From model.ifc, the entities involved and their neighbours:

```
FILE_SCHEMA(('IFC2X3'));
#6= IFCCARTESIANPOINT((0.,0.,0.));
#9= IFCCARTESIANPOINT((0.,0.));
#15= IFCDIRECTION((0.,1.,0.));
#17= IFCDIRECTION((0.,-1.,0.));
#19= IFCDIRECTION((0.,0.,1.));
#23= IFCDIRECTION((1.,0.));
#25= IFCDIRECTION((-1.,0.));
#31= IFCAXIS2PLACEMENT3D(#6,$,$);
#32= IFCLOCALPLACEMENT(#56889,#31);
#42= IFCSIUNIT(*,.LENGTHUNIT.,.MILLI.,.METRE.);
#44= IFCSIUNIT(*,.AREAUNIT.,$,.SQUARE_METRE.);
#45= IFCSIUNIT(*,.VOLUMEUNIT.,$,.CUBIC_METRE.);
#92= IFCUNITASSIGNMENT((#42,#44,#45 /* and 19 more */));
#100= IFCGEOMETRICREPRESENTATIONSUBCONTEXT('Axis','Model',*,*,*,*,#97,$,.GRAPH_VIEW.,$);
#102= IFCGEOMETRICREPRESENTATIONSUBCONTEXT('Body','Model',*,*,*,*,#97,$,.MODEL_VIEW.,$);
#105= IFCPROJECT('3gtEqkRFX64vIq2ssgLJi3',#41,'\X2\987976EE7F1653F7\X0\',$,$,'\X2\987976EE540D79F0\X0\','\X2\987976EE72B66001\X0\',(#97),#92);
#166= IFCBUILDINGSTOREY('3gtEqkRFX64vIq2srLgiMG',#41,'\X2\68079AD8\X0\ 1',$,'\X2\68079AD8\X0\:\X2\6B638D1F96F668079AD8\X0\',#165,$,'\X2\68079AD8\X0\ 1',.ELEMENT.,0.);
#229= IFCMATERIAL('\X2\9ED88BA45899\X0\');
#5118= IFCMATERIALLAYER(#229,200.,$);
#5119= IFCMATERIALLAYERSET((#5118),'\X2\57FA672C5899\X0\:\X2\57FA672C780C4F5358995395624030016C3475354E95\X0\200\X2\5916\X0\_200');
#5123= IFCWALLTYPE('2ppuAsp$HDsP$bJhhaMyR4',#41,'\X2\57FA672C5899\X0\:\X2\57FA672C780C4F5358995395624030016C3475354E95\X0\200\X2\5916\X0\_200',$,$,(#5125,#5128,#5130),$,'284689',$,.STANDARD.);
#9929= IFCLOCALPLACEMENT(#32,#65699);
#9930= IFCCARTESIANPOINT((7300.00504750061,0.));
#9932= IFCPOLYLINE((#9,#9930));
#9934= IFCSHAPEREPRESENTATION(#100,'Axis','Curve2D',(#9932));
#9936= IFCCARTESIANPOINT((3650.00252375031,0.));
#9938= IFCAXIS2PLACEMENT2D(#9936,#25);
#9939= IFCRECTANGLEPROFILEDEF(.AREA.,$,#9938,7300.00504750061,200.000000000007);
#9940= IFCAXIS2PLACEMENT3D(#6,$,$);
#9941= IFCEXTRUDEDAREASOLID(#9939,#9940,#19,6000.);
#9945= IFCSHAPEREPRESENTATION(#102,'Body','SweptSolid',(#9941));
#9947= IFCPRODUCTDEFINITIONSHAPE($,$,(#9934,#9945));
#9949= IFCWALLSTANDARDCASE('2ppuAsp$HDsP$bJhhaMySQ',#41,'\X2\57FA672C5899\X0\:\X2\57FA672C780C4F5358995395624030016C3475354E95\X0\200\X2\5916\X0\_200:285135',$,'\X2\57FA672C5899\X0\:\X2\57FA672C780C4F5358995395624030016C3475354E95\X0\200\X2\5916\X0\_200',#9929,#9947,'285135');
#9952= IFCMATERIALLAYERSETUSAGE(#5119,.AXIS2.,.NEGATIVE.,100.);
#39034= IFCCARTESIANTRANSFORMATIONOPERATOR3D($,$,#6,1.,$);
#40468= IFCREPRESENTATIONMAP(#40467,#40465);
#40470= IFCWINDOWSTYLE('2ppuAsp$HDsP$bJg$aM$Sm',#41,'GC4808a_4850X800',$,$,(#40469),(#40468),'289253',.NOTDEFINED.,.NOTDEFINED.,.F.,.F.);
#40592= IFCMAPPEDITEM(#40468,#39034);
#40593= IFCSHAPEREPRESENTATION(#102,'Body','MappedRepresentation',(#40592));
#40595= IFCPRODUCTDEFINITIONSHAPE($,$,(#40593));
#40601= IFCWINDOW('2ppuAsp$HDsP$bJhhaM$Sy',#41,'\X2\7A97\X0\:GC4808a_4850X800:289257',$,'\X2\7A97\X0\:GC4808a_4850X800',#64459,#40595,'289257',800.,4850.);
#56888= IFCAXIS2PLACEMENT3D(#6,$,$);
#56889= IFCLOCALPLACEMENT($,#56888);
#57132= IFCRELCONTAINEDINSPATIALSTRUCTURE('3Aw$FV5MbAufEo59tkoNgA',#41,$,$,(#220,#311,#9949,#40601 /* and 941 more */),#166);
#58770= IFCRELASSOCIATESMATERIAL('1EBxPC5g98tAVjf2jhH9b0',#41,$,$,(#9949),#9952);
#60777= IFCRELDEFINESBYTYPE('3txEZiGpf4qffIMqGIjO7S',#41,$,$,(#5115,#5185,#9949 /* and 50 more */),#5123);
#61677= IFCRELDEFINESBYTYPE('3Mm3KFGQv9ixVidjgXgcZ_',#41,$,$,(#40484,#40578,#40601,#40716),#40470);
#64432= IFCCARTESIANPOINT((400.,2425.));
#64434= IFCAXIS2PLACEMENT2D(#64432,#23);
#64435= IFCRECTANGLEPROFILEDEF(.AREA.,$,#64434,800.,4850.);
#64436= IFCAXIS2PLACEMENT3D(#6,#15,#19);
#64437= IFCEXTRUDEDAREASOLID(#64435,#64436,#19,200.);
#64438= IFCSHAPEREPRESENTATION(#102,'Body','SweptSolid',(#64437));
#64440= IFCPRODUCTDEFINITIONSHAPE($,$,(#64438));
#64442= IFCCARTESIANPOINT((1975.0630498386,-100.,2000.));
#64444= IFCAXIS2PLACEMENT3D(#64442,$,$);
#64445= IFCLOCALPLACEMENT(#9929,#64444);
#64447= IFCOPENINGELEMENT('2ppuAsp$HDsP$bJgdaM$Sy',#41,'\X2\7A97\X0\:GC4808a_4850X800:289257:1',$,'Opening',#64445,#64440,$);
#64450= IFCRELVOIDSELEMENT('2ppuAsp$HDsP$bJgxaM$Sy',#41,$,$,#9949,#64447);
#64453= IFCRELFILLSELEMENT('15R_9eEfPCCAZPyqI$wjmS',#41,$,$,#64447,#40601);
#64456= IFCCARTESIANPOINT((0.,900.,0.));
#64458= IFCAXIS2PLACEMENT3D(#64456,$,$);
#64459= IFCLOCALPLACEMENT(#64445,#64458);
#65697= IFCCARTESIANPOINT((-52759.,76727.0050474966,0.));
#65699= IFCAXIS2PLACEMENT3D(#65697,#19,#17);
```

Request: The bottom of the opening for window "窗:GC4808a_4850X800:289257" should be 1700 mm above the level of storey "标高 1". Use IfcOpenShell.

```python
import numpy as np
import ifcopenshell
import ifcopenshell.api.geometry
import ifcopenshell.geom
import ifcopenshell.util.element
import ifcopenshell.util.placement
import ifcopenshell.util.shape
import ifcopenshell.util.unit

model = ifcopenshell.open("model.ifc")
unit_scale = ifcopenshell.util.unit.calculate_unit_scale(model)

window = model.by_guid("2ppuAsp$HDsP$bJhhaM$Sy")
opening = window.FillsVoids[0].RelatingOpeningElement
storey = ifcopenshell.util.element.get_container(window, ifc_class="IfcBuildingStorey")
level = ifcopenshell.util.placement.get_local_placement(storey.ObjectPlacement)[2, 3]

# The opening's origin need not be at the sill, so measure its lowest point.
shape = ifcopenshell.geom.create_shape(ifcopenshell.geom.settings(), opening)
bottom = ifcopenshell.util.shape.get_shape_bottom_elevation(shape, shape.geometry) / unit_scale
dz = level + 1.7 / unit_scale - bottom

shift = np.array([0.0, 0.0, dz])
# The window is placed relative to its opening, so it follows when the opening moves.
matrix = ifcopenshell.util.placement.get_local_placement(opening.ObjectPlacement)
matrix[:3, 3] += shift
ifcopenshell.api.geometry.edit_object_placement(
    model, product=opening, matrix=matrix, is_si=False, should_transform_children=True
)

print(f"moved by {dz * unit_scale:+.3f} m")

model.write("model_updated.ifc")
```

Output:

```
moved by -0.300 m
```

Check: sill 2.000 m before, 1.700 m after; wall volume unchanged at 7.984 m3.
